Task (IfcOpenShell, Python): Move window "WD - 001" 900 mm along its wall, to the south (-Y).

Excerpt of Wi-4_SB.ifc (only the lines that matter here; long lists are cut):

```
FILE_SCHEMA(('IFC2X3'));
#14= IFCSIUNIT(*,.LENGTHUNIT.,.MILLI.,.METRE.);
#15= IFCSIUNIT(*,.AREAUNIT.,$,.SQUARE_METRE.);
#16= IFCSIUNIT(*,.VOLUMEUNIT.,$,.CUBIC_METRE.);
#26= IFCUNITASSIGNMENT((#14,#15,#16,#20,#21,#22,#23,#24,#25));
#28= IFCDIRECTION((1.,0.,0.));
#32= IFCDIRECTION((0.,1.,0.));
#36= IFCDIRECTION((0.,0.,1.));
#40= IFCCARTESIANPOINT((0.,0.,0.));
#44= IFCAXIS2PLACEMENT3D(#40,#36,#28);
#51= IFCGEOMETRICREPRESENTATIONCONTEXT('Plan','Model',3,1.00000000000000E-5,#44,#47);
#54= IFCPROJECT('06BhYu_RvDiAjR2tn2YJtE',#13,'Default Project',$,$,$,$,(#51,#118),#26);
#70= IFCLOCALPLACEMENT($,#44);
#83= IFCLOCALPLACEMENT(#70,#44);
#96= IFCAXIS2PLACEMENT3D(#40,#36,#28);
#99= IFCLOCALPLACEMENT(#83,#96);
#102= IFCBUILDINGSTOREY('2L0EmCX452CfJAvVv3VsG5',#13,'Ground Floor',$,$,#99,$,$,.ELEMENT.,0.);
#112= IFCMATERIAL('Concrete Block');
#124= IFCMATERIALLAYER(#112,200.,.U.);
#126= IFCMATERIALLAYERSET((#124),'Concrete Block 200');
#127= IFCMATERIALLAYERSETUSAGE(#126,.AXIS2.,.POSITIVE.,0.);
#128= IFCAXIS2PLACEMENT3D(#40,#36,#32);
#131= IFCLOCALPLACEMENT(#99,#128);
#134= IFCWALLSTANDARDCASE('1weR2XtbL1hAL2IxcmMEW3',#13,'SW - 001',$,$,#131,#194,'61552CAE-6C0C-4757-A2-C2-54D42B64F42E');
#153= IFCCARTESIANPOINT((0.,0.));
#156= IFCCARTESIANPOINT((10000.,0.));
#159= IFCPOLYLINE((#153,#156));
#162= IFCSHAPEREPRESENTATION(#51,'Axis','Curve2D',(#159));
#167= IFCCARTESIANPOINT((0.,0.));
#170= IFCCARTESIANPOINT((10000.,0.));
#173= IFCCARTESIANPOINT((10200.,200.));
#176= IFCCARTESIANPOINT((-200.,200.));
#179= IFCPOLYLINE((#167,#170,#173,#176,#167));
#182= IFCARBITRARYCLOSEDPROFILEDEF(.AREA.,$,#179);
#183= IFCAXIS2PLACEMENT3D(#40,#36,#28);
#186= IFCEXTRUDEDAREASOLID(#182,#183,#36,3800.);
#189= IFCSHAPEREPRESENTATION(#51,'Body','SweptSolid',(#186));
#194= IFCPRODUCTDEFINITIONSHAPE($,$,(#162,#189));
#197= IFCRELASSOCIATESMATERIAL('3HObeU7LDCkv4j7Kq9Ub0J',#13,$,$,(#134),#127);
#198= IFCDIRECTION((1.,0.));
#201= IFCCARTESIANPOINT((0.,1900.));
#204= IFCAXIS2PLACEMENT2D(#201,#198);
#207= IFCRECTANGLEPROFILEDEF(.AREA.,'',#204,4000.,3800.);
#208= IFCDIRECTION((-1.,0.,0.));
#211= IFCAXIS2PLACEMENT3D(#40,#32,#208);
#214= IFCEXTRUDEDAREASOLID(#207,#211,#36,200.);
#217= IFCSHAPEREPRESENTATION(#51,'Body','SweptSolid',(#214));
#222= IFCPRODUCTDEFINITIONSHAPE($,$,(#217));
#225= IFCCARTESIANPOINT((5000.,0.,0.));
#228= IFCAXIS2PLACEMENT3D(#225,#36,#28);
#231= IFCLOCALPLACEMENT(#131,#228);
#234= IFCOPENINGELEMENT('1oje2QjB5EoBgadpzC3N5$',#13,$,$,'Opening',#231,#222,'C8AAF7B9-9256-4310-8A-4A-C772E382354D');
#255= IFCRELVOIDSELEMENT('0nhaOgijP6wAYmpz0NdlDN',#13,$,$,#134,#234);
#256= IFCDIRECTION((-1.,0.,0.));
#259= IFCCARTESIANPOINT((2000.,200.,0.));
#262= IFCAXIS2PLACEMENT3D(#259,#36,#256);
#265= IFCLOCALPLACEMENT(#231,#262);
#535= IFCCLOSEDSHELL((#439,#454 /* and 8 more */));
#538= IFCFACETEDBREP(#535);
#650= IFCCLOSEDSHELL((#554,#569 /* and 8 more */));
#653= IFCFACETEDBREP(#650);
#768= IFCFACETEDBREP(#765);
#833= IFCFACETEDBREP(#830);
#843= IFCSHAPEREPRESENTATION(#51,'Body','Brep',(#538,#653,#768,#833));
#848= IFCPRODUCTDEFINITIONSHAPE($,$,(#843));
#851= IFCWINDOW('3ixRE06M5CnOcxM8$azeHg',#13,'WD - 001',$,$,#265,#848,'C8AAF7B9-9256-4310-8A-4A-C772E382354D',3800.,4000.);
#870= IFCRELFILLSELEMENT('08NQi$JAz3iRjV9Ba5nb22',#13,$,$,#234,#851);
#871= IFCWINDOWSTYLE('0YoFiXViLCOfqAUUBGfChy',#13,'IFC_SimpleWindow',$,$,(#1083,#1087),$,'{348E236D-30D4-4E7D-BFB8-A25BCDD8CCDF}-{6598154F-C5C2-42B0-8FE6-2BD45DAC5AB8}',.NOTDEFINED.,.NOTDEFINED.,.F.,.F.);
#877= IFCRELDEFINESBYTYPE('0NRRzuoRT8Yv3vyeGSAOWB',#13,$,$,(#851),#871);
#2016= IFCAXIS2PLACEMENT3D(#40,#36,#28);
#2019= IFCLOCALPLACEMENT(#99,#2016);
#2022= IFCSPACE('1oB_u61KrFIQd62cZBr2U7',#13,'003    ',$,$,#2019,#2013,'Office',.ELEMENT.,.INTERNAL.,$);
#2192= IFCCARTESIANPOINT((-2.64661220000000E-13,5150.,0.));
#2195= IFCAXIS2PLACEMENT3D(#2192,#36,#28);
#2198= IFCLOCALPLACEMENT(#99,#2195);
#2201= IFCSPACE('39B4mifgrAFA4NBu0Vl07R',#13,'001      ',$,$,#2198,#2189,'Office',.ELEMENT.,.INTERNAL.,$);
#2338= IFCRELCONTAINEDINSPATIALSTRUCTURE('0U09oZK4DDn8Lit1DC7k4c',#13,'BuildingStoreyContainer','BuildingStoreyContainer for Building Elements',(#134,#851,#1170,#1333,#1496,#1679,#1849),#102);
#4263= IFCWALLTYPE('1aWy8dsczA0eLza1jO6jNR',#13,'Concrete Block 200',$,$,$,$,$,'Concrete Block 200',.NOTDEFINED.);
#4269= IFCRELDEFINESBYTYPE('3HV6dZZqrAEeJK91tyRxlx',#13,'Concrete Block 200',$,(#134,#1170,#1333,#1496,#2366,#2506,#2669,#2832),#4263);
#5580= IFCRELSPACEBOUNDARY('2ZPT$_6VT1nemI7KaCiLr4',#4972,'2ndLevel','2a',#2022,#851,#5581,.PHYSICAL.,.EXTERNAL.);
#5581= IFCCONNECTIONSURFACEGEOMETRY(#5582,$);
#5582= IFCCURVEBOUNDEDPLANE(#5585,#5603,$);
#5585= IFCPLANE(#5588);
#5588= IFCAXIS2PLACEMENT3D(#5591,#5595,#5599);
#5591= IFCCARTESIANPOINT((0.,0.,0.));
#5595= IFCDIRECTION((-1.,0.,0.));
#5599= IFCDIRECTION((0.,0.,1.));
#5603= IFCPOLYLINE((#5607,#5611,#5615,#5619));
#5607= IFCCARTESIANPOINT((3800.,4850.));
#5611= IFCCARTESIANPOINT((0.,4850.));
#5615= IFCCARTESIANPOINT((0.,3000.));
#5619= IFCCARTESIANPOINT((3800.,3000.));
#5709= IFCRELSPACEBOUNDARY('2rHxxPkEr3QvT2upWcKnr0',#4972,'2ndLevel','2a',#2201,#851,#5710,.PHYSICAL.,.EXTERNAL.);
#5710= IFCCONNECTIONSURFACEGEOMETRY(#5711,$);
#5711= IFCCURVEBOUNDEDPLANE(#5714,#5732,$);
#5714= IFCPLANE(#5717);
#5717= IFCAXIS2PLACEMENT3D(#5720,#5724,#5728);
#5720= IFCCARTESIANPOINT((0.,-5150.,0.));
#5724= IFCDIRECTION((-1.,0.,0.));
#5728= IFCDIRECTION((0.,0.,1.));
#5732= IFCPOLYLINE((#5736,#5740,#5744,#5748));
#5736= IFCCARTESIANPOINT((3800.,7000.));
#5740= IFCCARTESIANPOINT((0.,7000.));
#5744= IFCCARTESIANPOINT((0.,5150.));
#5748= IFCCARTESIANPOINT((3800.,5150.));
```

```python
import numpy as np
import ifcopenshell
import ifcopenshell.api.geometry
import ifcopenshell.util.placement
import ifcopenshell.util.unit

model = ifcopenshell.open("Wi-4_SB.ifc")
unit_scale = ifcopenshell.util.unit.calculate_unit_scale(model)

window = model.by_id(851)
opening = window.FillsVoids[0].RelatingOpeningElement
wall = opening.VoidsElements[0].RelatingBuildingElement

wall_matrix = ifcopenshell.util.placement.get_local_placement(wall.ObjectPlacement)
shift = wall_matrix[:3, 0] * -0.9 / unit_scale
before = ifcopenshell.util.placement.get_local_placement(window.ObjectPlacement)[:3, 3].copy()

# The window is placed relative to its opening, so it follows when the opening moves.
matrix = ifcopenshell.util.placement.get_local_placement(opening.ObjectPlacement)
matrix[:3, 3] += shift
ifcopenshell.api.geometry.edit_object_placement(
    model, product=opening, matrix=matrix, is_si=False, should_transform_children=True
)

# Space boundary surfaces are stored in each space's coordinates; move them too.
for rel in window.ProvidesBoundaries:
    if not rel.ConnectionGeometry:
        continue
    surface = rel.ConnectionGeometry.SurfaceOnRelatingElement.BasisSurface
    space_matrix = ifcopenshell.util.placement.get_local_placement(rel.RelatingSpace.ObjectPlacement)
    point = np.array(surface.Position.Location.Coordinates) + space_matrix[:3, :3].T @ shift
    surface.Position = model.createIfcAxis2Placement3D(
        model.createIfcCartesianPoint(point.tolist()), surface.Position.Axis, surface.Position.RefDirection
    )

after = ifcopenshell.util.placement.get_local_placement(window.ObjectPlacement)[:3, 3]
print("window moved by", (after - before).round(3) + 0.0)

model.write("Wi-4_SB-out.ifc")
```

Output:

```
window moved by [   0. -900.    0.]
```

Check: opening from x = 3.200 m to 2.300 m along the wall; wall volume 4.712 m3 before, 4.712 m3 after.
